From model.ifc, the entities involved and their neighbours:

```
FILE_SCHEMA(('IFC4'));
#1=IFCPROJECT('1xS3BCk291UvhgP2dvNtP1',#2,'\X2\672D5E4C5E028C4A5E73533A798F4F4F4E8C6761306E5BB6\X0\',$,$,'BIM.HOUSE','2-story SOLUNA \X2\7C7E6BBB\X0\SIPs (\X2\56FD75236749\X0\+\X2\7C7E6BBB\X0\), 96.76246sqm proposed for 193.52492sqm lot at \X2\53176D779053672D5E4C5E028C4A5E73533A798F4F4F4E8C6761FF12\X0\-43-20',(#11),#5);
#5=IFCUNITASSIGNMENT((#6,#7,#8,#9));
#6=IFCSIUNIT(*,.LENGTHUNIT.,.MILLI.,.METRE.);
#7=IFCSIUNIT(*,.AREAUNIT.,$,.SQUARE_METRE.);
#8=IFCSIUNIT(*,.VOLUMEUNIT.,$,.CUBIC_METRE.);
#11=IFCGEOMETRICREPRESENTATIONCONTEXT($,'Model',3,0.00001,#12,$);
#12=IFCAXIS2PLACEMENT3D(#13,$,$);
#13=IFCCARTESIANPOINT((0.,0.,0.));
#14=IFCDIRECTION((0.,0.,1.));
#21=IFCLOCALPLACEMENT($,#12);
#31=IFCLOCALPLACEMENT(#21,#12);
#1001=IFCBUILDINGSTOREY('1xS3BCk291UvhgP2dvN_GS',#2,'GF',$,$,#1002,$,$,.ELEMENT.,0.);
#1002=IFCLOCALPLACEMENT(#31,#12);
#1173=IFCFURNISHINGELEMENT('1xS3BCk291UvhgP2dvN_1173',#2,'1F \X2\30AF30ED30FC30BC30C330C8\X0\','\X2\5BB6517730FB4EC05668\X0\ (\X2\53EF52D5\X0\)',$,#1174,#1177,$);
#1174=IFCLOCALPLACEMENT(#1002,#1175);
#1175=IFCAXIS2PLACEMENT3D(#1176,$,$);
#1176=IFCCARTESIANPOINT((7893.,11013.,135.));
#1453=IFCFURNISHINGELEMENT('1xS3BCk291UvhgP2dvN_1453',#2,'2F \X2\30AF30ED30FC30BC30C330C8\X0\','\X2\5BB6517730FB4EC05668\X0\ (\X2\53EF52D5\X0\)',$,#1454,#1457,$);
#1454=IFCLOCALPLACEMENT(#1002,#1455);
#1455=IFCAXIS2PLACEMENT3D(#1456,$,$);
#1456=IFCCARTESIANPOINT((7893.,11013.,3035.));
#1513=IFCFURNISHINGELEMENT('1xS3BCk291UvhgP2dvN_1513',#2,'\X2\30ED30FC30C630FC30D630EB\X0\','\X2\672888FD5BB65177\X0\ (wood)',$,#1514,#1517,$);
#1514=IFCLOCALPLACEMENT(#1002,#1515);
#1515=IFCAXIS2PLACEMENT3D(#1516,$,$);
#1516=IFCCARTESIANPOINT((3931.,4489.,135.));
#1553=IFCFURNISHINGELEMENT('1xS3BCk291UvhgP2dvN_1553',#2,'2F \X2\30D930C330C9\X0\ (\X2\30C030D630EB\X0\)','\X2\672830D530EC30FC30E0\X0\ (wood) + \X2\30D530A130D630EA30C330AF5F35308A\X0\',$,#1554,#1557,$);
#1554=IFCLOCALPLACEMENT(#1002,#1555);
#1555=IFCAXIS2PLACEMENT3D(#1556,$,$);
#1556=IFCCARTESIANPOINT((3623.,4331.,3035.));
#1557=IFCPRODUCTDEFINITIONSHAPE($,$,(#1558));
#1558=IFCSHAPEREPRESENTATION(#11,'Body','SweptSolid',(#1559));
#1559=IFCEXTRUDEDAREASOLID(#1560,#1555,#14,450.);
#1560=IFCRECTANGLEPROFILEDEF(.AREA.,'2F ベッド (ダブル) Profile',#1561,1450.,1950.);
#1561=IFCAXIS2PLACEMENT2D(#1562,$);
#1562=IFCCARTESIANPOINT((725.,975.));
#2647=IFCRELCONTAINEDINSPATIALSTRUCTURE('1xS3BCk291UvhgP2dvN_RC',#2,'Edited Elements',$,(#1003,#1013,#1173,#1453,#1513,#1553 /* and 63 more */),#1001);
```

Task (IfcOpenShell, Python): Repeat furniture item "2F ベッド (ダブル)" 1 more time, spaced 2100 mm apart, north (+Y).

```python
import numpy as np
import ifcopenshell
import ifcopenshell.api.geometry
import ifcopenshell.api.root
import ifcopenshell.util.element
import ifcopenshell.util.placement
import ifcopenshell.util.unit

model = ifcopenshell.open("model.ifc")
unit_scale = ifcopenshell.util.unit.calculate_unit_scale(model)


def reuse_history(source, copy):
    """copy_class also copies each property set's owner history, people and application; keep the originals."""
    for rel in copy.IsDefinedBy:
        if rel.is_a("IfcRelDefinesByProperties") and (history := rel.RelatingPropertyDefinition.OwnerHistory):
            rel.RelatingPropertyDefinition.OwnerHistory = source.OwnerHistory
            ifcopenshell.util.element.remove_deep2(model, history)


source = model.by_id(1553)
base = ifcopenshell.util.placement.get_local_placement(source.ObjectPlacement)
step = np.array([0.0, 1.0, 0.0]) * 2.1 / unit_scale

for i in range(1, 2):
    copy = ifcopenshell.api.root.copy_class(model, product=source)
    copy.Representation = ifcopenshell.util.element.copy_deep(
        model, source.Representation, exclude=["IfcGeometricRepresentationContext", "IfcRepresentationMap"]
    )
    reuse_history(source, copy)
    matrix = base.copy()
    matrix[:3, 3] += i * step
    print("added at", matrix[:3, 3].round(3) + 0.0)
    ifcopenshell.api.geometry.edit_object_placement(model, product=copy, matrix=matrix, is_si=False)

model.write("model_edited.ifc")
```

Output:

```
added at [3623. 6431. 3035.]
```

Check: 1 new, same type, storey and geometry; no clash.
